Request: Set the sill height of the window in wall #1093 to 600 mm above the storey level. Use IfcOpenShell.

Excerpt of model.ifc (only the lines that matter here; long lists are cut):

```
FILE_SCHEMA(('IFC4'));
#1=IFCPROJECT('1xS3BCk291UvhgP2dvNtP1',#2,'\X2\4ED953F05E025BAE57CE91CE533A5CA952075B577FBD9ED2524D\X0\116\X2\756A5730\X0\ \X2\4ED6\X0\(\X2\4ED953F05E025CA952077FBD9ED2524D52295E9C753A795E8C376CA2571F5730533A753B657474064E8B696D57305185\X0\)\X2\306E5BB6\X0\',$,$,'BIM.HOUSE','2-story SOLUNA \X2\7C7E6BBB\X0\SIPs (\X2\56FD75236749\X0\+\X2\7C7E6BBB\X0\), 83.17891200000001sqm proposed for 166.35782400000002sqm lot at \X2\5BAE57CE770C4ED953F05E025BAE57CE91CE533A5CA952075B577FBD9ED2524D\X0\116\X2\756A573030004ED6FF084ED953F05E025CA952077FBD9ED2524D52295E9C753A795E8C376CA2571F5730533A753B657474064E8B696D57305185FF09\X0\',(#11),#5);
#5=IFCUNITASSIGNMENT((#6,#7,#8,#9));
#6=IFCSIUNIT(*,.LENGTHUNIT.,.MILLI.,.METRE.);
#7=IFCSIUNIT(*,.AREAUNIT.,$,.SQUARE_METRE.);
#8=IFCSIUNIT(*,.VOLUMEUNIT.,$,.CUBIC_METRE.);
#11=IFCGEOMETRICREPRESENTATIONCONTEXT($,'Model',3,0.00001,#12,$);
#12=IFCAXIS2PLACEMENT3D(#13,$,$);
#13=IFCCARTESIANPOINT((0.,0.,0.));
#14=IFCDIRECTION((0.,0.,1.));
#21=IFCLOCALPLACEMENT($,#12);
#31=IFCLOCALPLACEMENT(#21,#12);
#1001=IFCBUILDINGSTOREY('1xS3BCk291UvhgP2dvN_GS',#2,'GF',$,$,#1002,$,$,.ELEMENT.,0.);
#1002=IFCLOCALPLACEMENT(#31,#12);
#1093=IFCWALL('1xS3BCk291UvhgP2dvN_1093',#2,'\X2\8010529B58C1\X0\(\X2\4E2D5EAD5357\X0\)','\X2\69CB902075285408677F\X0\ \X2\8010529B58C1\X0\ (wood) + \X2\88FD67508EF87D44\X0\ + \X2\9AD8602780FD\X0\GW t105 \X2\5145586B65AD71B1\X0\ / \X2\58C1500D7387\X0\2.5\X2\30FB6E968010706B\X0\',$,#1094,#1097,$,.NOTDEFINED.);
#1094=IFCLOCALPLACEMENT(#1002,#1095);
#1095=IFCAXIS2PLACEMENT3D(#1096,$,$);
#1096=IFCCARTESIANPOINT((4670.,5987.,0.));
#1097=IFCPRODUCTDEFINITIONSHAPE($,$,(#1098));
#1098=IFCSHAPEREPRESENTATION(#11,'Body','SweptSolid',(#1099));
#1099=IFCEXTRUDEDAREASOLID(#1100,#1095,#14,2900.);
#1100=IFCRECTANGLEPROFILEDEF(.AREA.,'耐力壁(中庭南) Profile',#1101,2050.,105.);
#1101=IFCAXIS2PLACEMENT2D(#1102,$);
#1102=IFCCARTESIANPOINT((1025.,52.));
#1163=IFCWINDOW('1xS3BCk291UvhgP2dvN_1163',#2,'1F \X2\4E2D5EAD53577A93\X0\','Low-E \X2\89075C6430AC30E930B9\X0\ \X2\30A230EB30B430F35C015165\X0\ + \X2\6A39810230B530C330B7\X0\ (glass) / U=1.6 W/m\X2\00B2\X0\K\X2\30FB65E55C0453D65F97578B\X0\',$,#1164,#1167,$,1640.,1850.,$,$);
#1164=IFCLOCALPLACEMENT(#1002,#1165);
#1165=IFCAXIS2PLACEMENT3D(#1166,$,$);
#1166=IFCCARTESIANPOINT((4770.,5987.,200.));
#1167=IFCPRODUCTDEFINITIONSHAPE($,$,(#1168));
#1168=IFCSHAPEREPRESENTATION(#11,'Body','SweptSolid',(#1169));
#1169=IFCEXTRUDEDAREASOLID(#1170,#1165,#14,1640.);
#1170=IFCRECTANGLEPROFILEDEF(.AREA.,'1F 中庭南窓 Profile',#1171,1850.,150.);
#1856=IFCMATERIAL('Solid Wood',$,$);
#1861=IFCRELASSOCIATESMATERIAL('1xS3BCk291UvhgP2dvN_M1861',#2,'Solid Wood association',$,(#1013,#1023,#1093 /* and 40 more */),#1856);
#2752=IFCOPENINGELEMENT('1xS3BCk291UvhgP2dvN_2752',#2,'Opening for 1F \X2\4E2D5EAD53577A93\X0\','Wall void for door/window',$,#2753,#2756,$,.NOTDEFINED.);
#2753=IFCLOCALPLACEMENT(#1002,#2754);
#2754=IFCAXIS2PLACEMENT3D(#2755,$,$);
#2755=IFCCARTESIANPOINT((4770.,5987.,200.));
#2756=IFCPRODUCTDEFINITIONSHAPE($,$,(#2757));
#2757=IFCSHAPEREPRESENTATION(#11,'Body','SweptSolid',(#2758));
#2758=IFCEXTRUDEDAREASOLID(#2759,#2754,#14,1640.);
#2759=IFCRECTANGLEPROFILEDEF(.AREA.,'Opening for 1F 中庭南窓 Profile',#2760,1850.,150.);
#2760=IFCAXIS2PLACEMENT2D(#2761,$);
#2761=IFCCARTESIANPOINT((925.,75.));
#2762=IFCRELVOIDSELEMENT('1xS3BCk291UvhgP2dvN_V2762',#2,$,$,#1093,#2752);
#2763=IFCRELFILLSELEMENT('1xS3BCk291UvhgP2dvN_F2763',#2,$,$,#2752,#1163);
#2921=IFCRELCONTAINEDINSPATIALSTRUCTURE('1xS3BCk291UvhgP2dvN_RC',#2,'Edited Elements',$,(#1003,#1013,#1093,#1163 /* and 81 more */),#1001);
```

```python
import numpy as np
import ifcopenshell
import ifcopenshell.api.geometry
import ifcopenshell.geom
import ifcopenshell.util.element
import ifcopenshell.util.placement
import ifcopenshell.util.shape
import ifcopenshell.util.unit

model = ifcopenshell.open("model.ifc")
unit_scale = ifcopenshell.util.unit.calculate_unit_scale(model)

window = model.by_id(1163)
opening = window.FillsVoids[0].RelatingOpeningElement
storey = ifcopenshell.util.element.get_container(window, ifc_class="IfcBuildingStorey")
level = ifcopenshell.util.placement.get_local_placement(storey.ObjectPlacement)[2, 3]

# The opening's origin need not be at the sill, so measure its lowest point.
shape = ifcopenshell.geom.create_shape(ifcopenshell.geom.settings(), opening)
bottom = ifcopenshell.util.shape.get_shape_bottom_elevation(shape, shape.geometry) / unit_scale
dz = level + 0.6 / unit_scale - bottom

shift = np.array([0.0, 0.0, dz])
# The window is not placed relative to its opening, so move both.
for product in (opening, window):
    matrix = ifcopenshell.util.placement.get_local_placement(product.ObjectPlacement)
    matrix[:3, 3] += shift
    ifcopenshell.api.geometry.edit_object_placement(model, product=product, matrix=matrix, is_si=False)

print(f"moved by {dz * unit_scale:+.3f} m")

model.write("model_v2.ifc")
```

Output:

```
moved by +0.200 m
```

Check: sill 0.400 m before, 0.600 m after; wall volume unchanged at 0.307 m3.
